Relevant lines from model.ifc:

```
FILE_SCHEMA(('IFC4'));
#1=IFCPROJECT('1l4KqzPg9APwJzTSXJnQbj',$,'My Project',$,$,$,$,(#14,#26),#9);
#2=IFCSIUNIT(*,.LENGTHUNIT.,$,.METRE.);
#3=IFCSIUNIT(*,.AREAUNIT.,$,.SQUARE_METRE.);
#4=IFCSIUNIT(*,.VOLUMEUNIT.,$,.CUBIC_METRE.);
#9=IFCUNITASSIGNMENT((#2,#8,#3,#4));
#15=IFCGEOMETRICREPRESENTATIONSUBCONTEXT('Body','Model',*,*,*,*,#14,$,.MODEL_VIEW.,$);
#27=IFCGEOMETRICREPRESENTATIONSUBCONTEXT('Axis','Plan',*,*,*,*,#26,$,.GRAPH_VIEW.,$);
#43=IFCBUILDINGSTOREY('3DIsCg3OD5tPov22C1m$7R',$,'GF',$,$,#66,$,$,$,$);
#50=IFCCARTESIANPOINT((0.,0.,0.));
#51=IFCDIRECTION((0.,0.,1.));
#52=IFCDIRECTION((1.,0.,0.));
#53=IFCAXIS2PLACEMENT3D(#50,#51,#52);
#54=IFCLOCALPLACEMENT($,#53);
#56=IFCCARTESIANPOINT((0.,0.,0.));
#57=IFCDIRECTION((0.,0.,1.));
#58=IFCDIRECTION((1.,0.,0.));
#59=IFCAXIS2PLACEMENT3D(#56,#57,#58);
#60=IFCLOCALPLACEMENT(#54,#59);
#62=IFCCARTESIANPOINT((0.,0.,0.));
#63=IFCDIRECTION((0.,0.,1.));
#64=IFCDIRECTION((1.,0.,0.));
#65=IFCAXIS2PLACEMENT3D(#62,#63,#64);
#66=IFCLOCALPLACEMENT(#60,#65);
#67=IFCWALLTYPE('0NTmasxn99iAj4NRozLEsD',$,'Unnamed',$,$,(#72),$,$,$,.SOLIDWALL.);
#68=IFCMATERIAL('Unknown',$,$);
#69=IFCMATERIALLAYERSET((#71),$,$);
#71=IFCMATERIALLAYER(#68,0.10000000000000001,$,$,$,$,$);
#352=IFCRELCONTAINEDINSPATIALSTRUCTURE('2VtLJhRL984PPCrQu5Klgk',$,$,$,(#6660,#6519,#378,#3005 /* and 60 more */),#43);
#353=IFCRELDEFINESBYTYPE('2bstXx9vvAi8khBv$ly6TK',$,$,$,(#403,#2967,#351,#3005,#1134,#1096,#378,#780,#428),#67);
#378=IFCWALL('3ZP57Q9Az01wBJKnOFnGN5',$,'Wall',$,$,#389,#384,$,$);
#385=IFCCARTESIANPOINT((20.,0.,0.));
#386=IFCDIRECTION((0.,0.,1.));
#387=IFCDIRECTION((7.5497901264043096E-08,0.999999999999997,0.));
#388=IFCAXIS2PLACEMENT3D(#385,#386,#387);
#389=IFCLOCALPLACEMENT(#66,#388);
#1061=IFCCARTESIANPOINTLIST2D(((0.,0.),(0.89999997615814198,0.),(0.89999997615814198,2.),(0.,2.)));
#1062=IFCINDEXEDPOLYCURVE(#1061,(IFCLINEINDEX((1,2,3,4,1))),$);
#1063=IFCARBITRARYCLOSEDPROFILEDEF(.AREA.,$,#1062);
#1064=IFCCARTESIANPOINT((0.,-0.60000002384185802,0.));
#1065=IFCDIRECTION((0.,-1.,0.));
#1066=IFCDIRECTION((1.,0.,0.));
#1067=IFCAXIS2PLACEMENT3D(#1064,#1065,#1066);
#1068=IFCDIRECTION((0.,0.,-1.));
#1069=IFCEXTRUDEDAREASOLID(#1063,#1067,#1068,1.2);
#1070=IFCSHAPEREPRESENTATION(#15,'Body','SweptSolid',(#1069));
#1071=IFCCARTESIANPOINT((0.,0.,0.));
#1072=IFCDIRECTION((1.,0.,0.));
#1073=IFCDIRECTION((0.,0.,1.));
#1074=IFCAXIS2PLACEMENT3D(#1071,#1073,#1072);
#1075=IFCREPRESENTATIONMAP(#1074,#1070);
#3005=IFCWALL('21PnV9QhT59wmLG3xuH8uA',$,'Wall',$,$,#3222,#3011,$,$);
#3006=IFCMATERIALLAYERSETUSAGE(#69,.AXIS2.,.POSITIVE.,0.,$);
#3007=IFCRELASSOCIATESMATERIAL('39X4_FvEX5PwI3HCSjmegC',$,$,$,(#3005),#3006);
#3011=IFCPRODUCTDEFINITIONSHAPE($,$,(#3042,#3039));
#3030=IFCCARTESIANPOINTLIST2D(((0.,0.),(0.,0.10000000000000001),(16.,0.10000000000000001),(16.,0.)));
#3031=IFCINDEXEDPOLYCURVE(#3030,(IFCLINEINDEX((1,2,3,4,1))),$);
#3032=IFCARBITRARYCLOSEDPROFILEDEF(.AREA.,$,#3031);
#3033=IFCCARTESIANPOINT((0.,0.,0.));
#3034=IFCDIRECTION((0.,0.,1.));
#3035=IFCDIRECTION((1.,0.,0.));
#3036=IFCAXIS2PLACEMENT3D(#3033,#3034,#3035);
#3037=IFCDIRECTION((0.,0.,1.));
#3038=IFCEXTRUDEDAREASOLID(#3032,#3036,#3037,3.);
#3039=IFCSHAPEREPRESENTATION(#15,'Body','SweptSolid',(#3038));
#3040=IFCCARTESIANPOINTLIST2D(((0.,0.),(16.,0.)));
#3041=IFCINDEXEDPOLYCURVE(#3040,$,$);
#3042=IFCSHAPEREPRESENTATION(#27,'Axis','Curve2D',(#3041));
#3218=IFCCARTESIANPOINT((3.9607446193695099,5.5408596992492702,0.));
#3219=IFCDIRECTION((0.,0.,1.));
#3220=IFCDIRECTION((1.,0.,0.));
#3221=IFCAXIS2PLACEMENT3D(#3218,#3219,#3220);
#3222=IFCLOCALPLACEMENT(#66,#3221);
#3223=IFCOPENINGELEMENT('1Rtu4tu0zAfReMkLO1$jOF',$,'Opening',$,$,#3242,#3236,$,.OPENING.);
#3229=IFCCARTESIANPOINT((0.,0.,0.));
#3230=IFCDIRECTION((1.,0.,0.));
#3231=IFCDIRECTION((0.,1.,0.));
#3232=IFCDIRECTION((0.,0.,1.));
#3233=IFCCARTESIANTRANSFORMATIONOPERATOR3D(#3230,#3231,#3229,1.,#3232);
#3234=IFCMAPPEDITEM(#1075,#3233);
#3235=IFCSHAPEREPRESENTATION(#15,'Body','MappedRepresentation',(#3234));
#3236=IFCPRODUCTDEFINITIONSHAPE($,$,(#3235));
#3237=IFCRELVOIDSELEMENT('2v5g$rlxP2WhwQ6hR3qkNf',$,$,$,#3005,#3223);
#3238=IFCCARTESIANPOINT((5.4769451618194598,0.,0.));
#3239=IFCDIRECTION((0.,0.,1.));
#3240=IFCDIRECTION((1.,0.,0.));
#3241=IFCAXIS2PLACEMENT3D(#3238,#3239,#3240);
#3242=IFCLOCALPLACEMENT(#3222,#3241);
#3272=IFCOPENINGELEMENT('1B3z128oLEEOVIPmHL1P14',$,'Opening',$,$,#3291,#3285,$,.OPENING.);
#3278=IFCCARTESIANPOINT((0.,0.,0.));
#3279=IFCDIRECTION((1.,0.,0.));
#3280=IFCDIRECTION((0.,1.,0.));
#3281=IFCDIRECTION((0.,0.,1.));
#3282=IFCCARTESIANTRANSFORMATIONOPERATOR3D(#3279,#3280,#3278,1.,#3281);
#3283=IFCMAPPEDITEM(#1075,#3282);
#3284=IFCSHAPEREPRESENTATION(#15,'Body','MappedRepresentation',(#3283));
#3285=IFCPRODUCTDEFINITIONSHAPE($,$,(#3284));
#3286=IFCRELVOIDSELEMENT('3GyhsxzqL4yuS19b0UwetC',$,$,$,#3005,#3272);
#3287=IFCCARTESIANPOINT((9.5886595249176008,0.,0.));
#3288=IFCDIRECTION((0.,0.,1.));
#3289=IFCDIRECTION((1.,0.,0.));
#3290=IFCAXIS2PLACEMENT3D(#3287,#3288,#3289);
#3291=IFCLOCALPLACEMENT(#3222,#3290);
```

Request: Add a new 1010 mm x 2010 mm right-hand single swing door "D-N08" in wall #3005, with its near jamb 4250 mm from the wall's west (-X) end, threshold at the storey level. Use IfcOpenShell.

```python
import numpy as np
import ifcopenshell
import ifcopenshell.api.feature
import ifcopenshell.api.geometry
import ifcopenshell.api.root
import ifcopenshell.api.spatial
import ifcopenshell.geom
import ifcopenshell.util.element
import ifcopenshell.util.placement
import ifcopenshell.util.representation
import ifcopenshell.util.shape
import ifcopenshell.util.unit

model = ifcopenshell.open("model.ifc")
unit_scale = ifcopenshell.util.unit.calculate_unit_scale(model)
settings = ifcopenshell.geom.settings()


def volume(element):
    """Net volume in cubic metres, openings subtracted."""
    shape = ifcopenshell.geom.create_shape(settings, element)
    return ifcopenshell.util.shape.get_volume(shape.geometry)


wall = model.by_id(3005)
storey = ifcopenshell.util.element.get_container(wall, ifc_class="IfcBuildingStorey")
context = ifcopenshell.util.representation.get_context(model, "Model", "Body", "MODEL_VIEW")
before = volume(wall)

width, height, from_end, sill = 1.01, 2.01, 4.25, 0.0  # metres

# The wall runs along its own X axis, and the end named is its -X end.
wall_shape = ifcopenshell.geom.create_shape(settings, wall)
x, y, z = ifcopenshell.util.shape.get_vertices(wall_shape.geometry).T
start = x.min() + from_end
face, thickness = float(y.min()), float(y.max() - y.min())
wall_matrix = ifcopenshell.util.placement.get_local_placement(wall.ObjectPlacement)
level = ifcopenshell.util.placement.get_local_placement(storey.ObjectPlacement)[2, 3]


def in_wall(x, y):
    """Placement at x, y metres in the wall's axes, at sill height."""
    matrix = wall_matrix.copy()
    matrix[:, 3] = wall_matrix @ np.array([x / unit_scale, y / unit_scale, 0.0, 1.0])
    matrix[2, 3] = level + sill / unit_scale
    return matrix


# Opening: a box that overshoots both wall faces by 50 mm.
opening = ifcopenshell.api.root.create_entity(model, ifc_class="IfcOpeningElement", predefined_type="OPENING")
box = ifcopenshell.api.geometry.add_wall_representation(
    model, context=context, length=width, height=height, thickness=thickness + 0.1
)
ifcopenshell.api.geometry.assign_representation(model, product=opening, representation=box)
ifcopenshell.api.geometry.edit_object_placement(model, product=opening, matrix=in_wall(start, face - 0.05), is_si=False)
ifcopenshell.api.feature.add_feature(model, feature=opening, element=wall)

door = ifcopenshell.api.root.create_entity(model, ifc_class="IfcDoor", name="D-N08", predefined_type="DOOR")
door.OverallWidth, door.OverallHeight = width / unit_scale, height / unit_scale
door.OperationType = "SINGLE_SWING_RIGHT"
body = ifcopenshell.api.geometry.add_door_representation(
    model,
    context=context,
    overall_width=door.OverallWidth,
    overall_height=door.OverallHeight,
    operation_type="SINGLE_SWING_RIGHT",
    lining_properties={"LiningDepth": thickness / unit_scale, "ThresholdDepth": thickness / unit_scale},
)
ifcopenshell.api.geometry.assign_representation(model, product=door, representation=body)
ifcopenshell.api.spatial.assign_container(model, products=[door], relating_structure=storey)
ifcopenshell.api.feature.add_filling(model, opening=opening, element=door)

# The lining spans the wall, so the door starts at the wall face.
ifcopenshell.api.geometry.edit_object_placement(model, product=door, matrix=in_wall(start, face), is_si=False)

after = volume(wall)

print(f"wall volume {before:.3f} -> {after:.3f} m3")

model.write("model_updated.ifc")
```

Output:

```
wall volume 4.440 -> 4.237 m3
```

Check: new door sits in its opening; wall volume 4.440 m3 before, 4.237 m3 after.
